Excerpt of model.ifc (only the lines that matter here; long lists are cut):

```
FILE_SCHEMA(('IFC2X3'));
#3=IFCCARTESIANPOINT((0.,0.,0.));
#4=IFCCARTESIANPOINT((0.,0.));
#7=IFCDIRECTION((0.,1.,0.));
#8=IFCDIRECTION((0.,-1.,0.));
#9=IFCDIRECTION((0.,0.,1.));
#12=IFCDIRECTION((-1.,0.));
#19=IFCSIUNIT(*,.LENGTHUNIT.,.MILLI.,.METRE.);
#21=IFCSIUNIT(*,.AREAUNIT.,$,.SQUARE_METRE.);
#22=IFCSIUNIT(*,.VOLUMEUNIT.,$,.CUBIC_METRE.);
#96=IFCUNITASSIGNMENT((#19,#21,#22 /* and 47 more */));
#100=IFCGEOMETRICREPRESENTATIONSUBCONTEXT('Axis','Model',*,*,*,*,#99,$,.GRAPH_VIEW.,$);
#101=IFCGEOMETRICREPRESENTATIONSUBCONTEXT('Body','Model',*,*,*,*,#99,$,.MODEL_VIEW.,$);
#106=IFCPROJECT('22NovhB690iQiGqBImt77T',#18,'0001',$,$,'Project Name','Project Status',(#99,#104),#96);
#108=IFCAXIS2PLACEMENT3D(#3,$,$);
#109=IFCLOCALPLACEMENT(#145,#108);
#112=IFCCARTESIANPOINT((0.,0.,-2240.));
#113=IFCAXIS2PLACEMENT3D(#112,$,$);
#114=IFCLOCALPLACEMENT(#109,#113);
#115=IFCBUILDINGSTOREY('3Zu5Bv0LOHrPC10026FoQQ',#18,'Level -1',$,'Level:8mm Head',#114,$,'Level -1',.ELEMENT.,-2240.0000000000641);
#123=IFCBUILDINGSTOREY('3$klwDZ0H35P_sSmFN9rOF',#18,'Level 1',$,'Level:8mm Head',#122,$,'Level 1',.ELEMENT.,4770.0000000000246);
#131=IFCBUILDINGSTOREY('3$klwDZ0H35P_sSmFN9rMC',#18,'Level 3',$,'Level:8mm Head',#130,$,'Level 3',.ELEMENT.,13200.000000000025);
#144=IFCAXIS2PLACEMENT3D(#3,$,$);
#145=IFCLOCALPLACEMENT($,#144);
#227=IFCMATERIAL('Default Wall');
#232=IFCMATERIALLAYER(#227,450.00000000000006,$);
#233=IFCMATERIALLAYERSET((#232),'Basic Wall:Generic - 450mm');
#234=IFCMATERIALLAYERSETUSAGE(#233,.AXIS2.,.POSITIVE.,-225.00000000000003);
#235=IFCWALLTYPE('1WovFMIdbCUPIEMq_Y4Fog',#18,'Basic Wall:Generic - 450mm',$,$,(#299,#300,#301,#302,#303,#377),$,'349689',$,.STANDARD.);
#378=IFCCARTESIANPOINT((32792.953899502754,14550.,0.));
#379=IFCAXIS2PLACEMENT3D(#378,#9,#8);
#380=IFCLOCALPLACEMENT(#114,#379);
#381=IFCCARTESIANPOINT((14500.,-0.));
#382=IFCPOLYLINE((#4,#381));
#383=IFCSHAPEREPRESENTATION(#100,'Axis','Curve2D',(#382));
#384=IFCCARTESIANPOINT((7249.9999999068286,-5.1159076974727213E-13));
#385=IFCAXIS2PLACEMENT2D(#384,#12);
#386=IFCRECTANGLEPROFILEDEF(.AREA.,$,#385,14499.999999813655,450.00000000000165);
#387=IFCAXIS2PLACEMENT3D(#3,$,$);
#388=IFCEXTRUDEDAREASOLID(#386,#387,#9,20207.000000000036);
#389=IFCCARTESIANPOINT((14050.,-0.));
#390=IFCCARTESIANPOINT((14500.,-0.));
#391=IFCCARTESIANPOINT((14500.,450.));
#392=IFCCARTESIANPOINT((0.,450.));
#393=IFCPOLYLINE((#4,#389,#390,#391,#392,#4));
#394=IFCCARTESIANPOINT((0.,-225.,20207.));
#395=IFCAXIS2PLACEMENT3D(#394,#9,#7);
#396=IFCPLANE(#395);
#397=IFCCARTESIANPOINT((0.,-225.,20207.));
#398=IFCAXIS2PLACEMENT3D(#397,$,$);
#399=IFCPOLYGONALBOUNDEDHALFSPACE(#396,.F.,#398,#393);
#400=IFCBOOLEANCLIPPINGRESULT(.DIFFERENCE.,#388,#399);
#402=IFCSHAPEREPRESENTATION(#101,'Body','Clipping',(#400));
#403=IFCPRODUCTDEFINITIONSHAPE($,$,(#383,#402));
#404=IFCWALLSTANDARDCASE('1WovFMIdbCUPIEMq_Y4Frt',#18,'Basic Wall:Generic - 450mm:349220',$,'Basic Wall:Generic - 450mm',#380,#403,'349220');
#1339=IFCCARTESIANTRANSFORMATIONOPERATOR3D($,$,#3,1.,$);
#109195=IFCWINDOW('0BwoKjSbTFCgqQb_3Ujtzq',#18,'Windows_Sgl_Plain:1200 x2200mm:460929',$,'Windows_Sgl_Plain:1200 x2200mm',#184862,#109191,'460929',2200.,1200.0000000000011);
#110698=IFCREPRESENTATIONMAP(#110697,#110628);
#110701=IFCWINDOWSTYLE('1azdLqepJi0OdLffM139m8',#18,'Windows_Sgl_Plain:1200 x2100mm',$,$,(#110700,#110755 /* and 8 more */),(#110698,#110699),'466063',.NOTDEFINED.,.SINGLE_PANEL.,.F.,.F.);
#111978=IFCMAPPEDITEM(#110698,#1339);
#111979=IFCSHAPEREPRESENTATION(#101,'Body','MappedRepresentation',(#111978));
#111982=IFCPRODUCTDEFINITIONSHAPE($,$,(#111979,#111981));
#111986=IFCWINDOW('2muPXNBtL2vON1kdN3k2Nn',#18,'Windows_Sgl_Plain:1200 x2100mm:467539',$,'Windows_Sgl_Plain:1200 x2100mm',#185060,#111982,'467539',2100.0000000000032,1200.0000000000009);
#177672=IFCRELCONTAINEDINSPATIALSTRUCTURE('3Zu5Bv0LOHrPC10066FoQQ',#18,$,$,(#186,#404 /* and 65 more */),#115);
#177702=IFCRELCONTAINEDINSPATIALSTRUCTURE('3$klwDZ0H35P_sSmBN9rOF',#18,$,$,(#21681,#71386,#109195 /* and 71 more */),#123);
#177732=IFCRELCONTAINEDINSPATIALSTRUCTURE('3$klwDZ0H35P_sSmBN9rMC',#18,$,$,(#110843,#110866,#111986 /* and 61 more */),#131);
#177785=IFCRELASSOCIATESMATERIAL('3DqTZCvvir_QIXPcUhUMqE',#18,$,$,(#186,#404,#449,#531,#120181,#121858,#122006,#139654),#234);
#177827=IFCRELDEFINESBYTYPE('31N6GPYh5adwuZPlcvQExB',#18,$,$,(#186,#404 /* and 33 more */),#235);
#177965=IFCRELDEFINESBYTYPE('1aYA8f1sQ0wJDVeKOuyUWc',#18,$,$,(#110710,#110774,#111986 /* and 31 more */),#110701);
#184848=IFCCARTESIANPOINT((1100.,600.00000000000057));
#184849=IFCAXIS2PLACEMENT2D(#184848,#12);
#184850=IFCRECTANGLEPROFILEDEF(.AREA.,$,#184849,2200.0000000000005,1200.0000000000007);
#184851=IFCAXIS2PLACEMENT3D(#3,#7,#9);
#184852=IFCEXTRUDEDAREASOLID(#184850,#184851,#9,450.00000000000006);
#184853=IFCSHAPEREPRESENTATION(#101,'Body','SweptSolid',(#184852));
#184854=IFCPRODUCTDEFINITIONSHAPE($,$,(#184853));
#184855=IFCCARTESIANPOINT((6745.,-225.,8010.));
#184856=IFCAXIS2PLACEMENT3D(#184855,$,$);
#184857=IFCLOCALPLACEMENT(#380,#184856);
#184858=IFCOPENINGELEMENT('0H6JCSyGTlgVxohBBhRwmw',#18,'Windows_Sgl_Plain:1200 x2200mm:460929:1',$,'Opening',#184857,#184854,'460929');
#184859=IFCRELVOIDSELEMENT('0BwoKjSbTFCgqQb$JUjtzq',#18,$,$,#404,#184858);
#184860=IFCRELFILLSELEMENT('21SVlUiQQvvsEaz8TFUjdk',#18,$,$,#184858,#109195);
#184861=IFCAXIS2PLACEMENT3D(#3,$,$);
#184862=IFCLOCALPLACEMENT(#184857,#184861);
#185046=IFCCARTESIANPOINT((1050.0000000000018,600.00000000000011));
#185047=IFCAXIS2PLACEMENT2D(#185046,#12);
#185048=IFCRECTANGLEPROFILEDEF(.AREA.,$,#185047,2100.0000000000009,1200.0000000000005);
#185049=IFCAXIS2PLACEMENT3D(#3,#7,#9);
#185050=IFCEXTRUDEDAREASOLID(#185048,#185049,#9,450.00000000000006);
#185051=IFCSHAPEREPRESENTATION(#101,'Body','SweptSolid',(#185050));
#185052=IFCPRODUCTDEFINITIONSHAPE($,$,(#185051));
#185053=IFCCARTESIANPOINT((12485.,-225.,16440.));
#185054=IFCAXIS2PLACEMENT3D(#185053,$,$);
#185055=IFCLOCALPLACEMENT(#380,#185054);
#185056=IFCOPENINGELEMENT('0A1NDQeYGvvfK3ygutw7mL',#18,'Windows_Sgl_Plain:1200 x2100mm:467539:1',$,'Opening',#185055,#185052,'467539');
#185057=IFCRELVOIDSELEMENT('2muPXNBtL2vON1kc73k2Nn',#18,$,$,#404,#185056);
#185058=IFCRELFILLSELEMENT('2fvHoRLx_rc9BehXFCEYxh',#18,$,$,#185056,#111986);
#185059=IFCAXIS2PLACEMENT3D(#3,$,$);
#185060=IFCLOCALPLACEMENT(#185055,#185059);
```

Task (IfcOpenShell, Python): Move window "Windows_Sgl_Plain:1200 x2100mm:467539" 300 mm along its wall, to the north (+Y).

```python
import ifcopenshell
import ifcopenshell.api.geometry
import ifcopenshell.util.placement

model = ifcopenshell.open("model.ifc")

window = model.by_id(111986)
opening = window.FillsVoids[0].RelatingOpeningElement
wall = opening.VoidsElements[0].RelatingBuildingElement

wall_matrix = ifcopenshell.util.placement.get_local_placement(wall.ObjectPlacement)
shift = wall_matrix[:3, 0] * -300.0
before = ifcopenshell.util.placement.get_local_placement(window.ObjectPlacement)[:3, 3].copy()

# The window is placed relative to its opening, so it follows when the opening moves.
matrix = ifcopenshell.util.placement.get_local_placement(opening.ObjectPlacement)
matrix[:3, 3] += shift
ifcopenshell.api.geometry.edit_object_placement(
    model, product=opening, matrix=matrix, is_si=False, should_transform_children=True
)

after = ifcopenshell.util.placement.get_local_placement(window.ObjectPlacement)[:3, 3]
print("window moved by", (after - before).round(3) + 0.0)

model.write("model_edited.ifc")
```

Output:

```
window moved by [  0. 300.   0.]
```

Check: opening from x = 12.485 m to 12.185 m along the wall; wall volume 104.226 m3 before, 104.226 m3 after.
